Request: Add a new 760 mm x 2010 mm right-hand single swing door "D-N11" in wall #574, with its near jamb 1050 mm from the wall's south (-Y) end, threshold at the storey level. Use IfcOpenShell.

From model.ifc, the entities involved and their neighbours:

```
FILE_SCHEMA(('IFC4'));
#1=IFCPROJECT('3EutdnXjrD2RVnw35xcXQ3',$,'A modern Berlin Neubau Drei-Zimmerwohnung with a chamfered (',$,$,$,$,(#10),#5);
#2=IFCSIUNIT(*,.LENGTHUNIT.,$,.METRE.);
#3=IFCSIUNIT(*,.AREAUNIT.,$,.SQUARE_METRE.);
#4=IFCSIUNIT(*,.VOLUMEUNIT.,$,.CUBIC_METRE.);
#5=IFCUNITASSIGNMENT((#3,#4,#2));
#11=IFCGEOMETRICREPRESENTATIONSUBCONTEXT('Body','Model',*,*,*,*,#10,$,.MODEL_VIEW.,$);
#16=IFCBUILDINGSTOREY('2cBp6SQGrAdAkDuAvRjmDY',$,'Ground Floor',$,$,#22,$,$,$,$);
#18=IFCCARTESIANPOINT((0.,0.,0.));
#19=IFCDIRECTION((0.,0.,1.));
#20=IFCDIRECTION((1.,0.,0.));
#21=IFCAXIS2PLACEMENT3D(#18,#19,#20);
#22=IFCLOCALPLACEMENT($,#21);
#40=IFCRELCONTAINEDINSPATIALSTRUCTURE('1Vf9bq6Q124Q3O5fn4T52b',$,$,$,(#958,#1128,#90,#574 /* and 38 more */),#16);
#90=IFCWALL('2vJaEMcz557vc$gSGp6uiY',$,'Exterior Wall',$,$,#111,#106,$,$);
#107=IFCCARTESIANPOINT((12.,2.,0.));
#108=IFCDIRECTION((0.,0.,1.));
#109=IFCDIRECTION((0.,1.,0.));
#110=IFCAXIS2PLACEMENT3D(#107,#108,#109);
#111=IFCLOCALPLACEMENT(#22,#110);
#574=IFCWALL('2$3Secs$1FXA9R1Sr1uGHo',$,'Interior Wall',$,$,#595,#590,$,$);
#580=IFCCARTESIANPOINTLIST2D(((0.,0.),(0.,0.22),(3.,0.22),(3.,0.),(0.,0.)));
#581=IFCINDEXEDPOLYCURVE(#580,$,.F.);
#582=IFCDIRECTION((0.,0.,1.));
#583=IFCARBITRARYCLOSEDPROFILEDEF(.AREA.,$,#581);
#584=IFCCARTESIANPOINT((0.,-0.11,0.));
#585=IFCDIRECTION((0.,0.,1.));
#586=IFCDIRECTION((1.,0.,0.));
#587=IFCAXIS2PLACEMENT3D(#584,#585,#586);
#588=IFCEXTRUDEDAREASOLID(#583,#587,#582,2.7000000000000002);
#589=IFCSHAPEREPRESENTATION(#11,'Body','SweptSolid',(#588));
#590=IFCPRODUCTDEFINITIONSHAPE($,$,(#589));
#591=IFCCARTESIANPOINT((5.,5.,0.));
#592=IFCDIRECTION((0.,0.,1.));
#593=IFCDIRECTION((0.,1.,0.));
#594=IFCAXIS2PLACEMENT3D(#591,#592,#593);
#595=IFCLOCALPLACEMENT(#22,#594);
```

```python
import numpy as np
import ifcopenshell
import ifcopenshell.api.feature
import ifcopenshell.api.geometry
import ifcopenshell.api.root
import ifcopenshell.api.spatial
import ifcopenshell.geom
import ifcopenshell.util.element
import ifcopenshell.util.placement
import ifcopenshell.util.representation
import ifcopenshell.util.shape
import ifcopenshell.util.unit

model = ifcopenshell.open("model.ifc")
unit_scale = ifcopenshell.util.unit.calculate_unit_scale(model)
settings = ifcopenshell.geom.settings()


def volume(element):
    """Net volume in cubic metres, openings subtracted."""
    shape = ifcopenshell.geom.create_shape(settings, element)
    return ifcopenshell.util.shape.get_volume(shape.geometry)


wall = model.by_id(574)
storey = ifcopenshell.util.element.get_container(wall, ifc_class="IfcBuildingStorey")
context = ifcopenshell.util.representation.get_context(model, "Model", "Body", "MODEL_VIEW")
before = volume(wall)

width, height, from_end, sill = 0.76, 2.01, 1.05, 0.0  # metres

# The wall runs along its own X axis, and the end named is its -X end.
wall_shape = ifcopenshell.geom.create_shape(settings, wall)
x, y, z = ifcopenshell.util.shape.get_vertices(wall_shape.geometry).T
start = x.min() + from_end
face, thickness = float(y.min()), float(y.max() - y.min())
wall_matrix = ifcopenshell.util.placement.get_local_placement(wall.ObjectPlacement)
level = ifcopenshell.util.placement.get_local_placement(storey.ObjectPlacement)[2, 3]


def in_wall(x, y):
    """Placement at x, y metres in the wall's axes, at sill height."""
    matrix = wall_matrix.copy()
    matrix[:, 3] = wall_matrix @ np.array([x / unit_scale, y / unit_scale, 0.0, 1.0])
    matrix[2, 3] = level + sill / unit_scale
    return matrix


# Opening: a box that overshoots both wall faces by 50 mm.
opening = ifcopenshell.api.root.create_entity(model, ifc_class="IfcOpeningElement", predefined_type="OPENING")
box = ifcopenshell.api.geometry.add_wall_representation(
    model, context=context, length=width, height=height, thickness=thickness + 0.1
)
ifcopenshell.api.geometry.assign_representation(model, product=opening, representation=box)
ifcopenshell.api.geometry.edit_object_placement(model, product=opening, matrix=in_wall(start, face - 0.05), is_si=False)
ifcopenshell.api.feature.add_feature(model, feature=opening, element=wall)

door = ifcopenshell.api.root.create_entity(model, ifc_class="IfcDoor", name="D-N11", predefined_type="DOOR")
door.OverallWidth, door.OverallHeight = width / unit_scale, height / unit_scale
door.OperationType = "SINGLE_SWING_RIGHT"
body = ifcopenshell.api.geometry.add_door_representation(
    model,
    context=context,
    overall_width=door.OverallWidth,
    overall_height=door.OverallHeight,
    operation_type="SINGLE_SWING_RIGHT",
    lining_properties={"LiningDepth": thickness / unit_scale, "ThresholdDepth": thickness / unit_scale},
)
ifcopenshell.api.geometry.assign_representation(model, product=door, representation=body)
ifcopenshell.api.spatial.assign_container(model, products=[door], relating_structure=storey)
ifcopenshell.api.feature.add_filling(model, opening=opening, element=door)

# The lining spans the wall, so the door starts at the wall face.
ifcopenshell.api.geometry.edit_object_placement(model, product=door, matrix=in_wall(start, face), is_si=False)

after = volume(wall)

print(f"wall volume {before:.3f} -> {after:.3f} m3")

model.write("model_v2.ifc")
```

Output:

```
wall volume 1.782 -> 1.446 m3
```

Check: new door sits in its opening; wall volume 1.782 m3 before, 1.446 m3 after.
